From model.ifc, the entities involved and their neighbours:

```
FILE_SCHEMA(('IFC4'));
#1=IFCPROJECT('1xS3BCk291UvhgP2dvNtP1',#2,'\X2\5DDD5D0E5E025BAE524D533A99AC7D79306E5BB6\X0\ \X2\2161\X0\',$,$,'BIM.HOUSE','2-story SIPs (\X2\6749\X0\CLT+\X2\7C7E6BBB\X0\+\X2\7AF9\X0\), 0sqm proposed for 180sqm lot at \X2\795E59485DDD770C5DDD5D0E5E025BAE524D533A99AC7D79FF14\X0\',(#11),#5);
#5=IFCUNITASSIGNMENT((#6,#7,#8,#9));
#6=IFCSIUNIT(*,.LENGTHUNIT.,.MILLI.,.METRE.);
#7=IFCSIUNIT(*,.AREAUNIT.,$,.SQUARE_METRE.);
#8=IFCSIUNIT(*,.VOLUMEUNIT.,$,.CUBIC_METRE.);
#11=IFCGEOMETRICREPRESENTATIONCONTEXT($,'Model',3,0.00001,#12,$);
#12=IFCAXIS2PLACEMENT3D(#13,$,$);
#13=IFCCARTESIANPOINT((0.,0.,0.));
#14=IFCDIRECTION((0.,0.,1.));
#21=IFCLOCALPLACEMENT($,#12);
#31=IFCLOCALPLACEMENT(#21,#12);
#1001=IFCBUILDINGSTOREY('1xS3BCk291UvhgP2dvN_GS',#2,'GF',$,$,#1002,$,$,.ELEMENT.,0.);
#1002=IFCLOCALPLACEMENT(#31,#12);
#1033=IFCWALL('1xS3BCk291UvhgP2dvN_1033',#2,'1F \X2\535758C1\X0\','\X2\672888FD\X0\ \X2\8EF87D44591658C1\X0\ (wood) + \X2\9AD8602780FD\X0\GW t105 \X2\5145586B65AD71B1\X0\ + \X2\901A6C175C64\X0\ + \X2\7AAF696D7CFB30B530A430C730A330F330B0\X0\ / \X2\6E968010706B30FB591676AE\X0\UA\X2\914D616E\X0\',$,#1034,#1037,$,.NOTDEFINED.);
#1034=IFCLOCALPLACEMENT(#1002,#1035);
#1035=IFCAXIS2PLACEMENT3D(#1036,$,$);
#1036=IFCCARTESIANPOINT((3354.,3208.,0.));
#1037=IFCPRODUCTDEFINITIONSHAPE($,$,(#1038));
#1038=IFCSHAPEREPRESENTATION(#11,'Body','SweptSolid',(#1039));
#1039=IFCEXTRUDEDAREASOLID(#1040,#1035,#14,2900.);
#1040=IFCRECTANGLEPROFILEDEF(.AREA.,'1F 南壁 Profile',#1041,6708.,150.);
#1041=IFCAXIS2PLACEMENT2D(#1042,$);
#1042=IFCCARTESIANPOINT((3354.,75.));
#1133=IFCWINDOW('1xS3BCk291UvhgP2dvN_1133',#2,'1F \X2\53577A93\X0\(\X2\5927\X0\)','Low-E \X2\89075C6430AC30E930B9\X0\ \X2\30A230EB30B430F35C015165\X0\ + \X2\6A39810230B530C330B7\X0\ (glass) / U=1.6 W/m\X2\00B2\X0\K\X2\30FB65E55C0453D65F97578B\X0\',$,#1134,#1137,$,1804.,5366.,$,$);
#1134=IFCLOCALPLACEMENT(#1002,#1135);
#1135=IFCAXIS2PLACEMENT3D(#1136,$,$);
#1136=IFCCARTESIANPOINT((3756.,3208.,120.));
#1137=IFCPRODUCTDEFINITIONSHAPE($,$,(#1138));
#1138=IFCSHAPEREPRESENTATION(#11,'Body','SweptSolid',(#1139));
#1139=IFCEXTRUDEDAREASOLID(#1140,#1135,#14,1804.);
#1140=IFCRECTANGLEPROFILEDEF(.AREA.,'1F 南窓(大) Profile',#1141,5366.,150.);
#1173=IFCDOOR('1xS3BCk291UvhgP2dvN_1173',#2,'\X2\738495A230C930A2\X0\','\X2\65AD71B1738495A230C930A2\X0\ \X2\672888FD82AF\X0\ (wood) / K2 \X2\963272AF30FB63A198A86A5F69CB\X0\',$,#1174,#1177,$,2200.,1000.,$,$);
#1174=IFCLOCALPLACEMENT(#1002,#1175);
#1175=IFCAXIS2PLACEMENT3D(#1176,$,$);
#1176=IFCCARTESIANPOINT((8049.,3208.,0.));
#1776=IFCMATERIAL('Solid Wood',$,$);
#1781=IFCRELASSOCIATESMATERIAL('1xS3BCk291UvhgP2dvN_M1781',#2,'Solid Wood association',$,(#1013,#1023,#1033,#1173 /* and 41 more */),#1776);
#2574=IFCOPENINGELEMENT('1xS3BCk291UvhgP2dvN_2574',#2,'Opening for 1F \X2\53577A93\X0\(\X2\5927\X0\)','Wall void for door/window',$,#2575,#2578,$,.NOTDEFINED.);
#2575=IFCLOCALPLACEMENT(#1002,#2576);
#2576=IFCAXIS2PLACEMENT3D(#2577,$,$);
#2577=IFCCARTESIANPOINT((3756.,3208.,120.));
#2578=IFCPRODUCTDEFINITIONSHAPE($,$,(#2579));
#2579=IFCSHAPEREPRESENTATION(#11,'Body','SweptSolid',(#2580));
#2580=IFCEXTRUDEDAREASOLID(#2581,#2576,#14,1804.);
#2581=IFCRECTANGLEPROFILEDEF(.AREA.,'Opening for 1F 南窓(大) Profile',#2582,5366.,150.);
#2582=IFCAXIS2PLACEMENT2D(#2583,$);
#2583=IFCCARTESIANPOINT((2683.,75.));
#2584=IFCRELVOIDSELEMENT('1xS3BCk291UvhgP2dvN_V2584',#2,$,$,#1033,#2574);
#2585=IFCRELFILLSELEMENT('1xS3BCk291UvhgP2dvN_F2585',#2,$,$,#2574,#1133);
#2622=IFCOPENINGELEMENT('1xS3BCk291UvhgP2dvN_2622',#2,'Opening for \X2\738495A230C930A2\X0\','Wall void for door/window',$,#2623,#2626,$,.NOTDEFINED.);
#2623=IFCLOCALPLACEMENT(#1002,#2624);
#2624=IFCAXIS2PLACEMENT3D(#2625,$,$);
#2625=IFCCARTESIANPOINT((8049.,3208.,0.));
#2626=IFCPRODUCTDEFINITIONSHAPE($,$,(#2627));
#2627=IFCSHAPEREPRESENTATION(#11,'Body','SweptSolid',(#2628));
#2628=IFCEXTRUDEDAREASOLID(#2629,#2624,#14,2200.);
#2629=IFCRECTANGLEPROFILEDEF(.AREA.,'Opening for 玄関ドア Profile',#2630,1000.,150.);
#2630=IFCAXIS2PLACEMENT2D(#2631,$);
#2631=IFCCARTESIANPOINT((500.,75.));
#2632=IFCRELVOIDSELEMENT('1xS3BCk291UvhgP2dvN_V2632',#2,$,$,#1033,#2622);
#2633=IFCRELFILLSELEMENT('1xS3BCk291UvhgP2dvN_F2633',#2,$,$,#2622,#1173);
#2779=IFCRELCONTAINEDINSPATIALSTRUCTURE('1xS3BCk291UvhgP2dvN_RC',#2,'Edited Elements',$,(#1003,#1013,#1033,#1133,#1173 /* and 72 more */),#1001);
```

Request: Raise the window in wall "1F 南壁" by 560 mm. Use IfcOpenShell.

```python
import numpy as np
import ifcopenshell
import ifcopenshell.api.geometry
import ifcopenshell.util.placement
import ifcopenshell.util.unit

model = ifcopenshell.open("model.ifc")
unit_scale = ifcopenshell.util.unit.calculate_unit_scale(model)

window = model.by_guid("1xS3BCk291UvhgP2dvN_1133")
opening = window.FillsVoids[0].RelatingOpeningElement
dz = 0.56 / unit_scale

shift = np.array([0.0, 0.0, dz])
# The window is not placed relative to its opening, so move both.
for product in (opening, window):
    matrix = ifcopenshell.util.placement.get_local_placement(product.ObjectPlacement)
    matrix[:3, 3] += shift
    ifcopenshell.api.geometry.edit_object_placement(model, product=product, matrix=matrix, is_si=False)

print(f"moved by {dz * unit_scale:+.3f} m")

model.write("model_v2.ifc")
```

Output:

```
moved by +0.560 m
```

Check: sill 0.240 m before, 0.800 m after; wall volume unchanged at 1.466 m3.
